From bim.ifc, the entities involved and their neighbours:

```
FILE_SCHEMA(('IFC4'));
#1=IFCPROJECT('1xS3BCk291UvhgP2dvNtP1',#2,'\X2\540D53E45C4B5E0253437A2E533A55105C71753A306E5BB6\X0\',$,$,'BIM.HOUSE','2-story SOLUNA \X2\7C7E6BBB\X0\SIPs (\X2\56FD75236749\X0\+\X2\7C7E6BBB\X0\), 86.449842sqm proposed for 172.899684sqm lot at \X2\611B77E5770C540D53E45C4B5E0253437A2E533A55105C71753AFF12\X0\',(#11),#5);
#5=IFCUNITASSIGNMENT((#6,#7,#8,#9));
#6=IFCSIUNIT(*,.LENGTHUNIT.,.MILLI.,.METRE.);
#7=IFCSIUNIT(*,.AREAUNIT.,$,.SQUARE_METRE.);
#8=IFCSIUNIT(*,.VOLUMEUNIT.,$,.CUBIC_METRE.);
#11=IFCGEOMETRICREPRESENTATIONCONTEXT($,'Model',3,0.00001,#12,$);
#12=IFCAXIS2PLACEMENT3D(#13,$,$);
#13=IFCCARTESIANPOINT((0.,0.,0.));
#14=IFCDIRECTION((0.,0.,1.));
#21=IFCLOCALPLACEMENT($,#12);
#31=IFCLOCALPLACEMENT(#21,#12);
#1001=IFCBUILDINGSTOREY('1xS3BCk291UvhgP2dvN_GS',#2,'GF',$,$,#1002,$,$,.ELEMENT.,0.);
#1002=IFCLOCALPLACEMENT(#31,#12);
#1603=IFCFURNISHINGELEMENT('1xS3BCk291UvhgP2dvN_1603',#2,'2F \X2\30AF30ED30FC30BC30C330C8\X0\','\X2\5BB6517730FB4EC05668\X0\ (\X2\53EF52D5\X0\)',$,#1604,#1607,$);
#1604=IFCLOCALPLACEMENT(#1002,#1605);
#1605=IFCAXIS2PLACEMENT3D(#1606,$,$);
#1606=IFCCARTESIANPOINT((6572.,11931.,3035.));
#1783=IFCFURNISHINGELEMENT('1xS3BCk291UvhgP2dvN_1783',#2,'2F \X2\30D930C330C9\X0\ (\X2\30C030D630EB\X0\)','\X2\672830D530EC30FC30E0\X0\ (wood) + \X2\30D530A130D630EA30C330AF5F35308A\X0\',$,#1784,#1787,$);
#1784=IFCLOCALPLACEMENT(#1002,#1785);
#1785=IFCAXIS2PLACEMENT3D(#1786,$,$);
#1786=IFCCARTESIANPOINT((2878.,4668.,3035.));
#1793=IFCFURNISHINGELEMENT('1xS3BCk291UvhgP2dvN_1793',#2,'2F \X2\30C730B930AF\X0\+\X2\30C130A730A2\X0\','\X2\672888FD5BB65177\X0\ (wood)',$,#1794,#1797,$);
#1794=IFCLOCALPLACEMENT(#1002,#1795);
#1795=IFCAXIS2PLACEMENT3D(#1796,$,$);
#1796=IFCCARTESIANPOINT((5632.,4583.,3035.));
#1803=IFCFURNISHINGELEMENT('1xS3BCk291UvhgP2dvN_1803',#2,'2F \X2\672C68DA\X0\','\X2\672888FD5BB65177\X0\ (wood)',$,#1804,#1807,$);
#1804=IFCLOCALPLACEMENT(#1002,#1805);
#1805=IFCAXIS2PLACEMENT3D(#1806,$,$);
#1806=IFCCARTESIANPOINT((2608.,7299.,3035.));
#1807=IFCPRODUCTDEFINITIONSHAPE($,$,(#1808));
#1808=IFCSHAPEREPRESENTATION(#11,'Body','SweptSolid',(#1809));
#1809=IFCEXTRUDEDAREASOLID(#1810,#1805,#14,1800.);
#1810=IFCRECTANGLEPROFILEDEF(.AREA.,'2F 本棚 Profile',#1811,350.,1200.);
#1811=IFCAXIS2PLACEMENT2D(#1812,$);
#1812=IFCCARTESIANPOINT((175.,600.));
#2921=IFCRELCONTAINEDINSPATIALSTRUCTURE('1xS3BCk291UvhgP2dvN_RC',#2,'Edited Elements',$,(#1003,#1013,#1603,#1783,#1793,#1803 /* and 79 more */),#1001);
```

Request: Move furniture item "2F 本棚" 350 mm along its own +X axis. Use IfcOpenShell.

```python
import ifcopenshell
import ifcopenshell.api.geometry
import ifcopenshell.util.placement

model = ifcopenshell.open("bim.ifc")

item = model.by_guid("1xS3BCk291UvhgP2dvN_1803")
matrix = ifcopenshell.util.placement.get_local_placement(item.ObjectPlacement)
matrix[:3, 3] += matrix[:3, 0] * 350.0
ifcopenshell.api.geometry.edit_object_placement(model, product=item, matrix=matrix, is_si=False)

print(ifcopenshell.util.placement.get_local_placement(item.ObjectPlacement).round(3) + 0.0)

model.write("bim_updated.ifc")
```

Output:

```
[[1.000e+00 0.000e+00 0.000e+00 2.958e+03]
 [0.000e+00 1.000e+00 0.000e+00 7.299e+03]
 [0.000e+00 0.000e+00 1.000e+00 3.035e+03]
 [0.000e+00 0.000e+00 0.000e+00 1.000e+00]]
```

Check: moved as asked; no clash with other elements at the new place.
